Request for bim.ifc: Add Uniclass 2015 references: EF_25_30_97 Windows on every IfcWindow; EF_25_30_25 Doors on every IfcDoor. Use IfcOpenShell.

First a look at what the model holds.

```python
import ifcopenshell

model = ifcopenshell.open("bim.ifc")
print(model.schema)
print("classifications:", [c.Name for c in model.by_type("IfcClassification")])
for ifc_class in ("IfcDoor", "IfcRoof", "IfcStair", "IfcWall", "IfcWindow"):
    print(ifc_class, len(model.by_type(ifc_class)))
```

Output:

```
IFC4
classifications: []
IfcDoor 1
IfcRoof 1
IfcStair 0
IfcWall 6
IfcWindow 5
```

```python
import ifcopenshell
import ifcopenshell.api.classification

model = ifcopenshell.open("bim.ifc")

system = ifcopenshell.api.classification.add_classification(model, classification="Uniclass 2015")

codes = {
    "IfcWindow": ("EF_25_30_97", "Windows"),
    "IfcDoor": ("EF_25_30_25", "Doors"),
}
for ifc_class, (code, name) in codes.items():
    products = model.by_type(ifc_class)
    ifcopenshell.api.classification.add_reference(
        model, products=products, classification=system, identification=code, name=name
    )
    print(code, len(products))

model.write("bim-out.ifc")
```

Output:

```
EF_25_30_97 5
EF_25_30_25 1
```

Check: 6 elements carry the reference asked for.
